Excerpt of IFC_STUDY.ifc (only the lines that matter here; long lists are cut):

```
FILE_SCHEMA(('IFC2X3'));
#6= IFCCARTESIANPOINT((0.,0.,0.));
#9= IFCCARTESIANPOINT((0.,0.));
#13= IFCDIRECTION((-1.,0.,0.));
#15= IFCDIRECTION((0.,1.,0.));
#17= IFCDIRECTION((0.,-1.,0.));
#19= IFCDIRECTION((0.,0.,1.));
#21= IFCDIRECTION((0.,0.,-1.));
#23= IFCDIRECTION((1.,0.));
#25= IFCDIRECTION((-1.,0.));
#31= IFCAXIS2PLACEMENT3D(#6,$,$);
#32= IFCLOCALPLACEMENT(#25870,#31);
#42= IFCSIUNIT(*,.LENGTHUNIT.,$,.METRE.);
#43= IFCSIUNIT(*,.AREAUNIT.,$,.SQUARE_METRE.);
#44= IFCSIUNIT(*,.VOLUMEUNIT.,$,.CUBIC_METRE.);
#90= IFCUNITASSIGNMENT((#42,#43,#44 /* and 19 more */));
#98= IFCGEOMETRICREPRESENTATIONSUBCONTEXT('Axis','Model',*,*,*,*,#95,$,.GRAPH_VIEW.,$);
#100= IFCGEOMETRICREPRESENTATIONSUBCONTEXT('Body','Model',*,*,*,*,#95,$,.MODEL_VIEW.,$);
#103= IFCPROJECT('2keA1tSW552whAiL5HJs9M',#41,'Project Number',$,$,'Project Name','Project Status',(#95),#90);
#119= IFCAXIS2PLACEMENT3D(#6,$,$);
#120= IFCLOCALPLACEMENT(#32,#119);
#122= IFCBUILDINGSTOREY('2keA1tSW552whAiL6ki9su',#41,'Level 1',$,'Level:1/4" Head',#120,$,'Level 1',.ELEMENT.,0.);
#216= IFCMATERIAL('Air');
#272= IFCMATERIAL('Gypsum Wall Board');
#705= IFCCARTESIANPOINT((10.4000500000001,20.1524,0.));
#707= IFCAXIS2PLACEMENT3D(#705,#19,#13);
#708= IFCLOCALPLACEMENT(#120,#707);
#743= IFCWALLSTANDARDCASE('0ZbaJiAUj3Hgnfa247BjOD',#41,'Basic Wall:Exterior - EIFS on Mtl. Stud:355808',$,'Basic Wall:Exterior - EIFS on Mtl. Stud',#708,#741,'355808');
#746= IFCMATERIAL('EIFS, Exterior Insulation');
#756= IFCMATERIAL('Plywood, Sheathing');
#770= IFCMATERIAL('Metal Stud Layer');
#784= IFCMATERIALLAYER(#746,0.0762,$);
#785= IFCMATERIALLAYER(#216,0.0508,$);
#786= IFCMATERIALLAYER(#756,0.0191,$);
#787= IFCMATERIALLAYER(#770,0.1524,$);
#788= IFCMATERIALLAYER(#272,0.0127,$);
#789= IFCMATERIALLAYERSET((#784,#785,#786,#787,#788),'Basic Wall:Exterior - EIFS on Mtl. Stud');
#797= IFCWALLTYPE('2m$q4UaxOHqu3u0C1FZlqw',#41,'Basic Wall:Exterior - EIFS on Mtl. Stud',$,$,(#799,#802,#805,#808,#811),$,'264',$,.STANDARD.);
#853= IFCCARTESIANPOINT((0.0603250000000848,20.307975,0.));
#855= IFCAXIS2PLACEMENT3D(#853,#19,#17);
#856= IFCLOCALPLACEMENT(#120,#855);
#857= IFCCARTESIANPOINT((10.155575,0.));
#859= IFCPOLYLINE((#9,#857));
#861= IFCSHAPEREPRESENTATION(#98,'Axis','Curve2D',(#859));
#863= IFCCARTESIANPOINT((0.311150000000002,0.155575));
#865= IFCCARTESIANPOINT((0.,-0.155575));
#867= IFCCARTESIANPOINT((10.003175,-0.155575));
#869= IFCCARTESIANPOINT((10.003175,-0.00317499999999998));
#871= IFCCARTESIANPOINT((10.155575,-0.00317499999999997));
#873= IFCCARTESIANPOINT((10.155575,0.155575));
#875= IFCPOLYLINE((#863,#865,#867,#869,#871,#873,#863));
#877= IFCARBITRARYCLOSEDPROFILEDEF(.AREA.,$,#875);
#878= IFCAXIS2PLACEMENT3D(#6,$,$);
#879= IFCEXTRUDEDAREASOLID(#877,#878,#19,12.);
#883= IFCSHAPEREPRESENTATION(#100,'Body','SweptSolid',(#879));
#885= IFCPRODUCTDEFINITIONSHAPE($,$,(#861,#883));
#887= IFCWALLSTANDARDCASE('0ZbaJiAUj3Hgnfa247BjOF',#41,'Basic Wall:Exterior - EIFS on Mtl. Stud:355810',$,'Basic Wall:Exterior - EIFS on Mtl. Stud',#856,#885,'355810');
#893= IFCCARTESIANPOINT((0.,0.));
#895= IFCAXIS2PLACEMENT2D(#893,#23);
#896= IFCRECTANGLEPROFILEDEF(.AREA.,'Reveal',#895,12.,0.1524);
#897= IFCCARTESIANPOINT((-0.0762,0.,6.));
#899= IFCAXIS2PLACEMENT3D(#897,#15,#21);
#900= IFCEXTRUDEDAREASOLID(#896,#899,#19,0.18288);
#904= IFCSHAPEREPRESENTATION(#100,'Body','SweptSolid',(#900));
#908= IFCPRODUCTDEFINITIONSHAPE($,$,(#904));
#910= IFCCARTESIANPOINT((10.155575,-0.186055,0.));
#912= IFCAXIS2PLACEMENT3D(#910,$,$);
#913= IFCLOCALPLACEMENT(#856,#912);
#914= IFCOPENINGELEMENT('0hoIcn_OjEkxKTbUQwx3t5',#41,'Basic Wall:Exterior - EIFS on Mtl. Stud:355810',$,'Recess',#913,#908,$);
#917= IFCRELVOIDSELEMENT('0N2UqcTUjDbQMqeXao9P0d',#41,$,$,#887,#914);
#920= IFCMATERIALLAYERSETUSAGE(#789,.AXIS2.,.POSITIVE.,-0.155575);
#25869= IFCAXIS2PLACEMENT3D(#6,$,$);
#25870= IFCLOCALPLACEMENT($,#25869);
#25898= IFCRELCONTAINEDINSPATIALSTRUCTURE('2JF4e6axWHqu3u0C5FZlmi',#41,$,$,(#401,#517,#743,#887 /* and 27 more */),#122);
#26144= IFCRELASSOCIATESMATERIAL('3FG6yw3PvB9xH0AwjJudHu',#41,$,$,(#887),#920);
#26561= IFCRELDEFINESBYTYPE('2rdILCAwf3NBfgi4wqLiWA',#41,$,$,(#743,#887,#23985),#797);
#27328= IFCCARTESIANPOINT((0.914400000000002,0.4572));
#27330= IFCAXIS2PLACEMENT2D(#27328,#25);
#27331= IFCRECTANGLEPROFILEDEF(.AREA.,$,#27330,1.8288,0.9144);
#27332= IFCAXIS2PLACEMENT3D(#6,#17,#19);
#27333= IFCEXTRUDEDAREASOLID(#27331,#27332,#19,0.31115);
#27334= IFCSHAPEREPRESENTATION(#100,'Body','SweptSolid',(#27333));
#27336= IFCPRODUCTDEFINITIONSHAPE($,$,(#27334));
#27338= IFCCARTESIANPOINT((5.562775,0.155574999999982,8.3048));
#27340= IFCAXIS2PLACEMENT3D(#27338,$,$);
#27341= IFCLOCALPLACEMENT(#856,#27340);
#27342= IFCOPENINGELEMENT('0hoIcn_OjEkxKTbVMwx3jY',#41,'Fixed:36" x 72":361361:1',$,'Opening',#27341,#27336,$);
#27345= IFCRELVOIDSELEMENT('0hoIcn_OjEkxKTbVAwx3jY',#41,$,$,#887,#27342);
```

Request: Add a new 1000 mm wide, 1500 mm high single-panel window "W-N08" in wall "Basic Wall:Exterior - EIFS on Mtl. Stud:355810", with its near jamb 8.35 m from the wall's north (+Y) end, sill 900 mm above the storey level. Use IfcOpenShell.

```python
import numpy as np
import ifcopenshell
import ifcopenshell.api.feature
import ifcopenshell.api.geometry
import ifcopenshell.api.root
import ifcopenshell.api.spatial
import ifcopenshell.api.type
import ifcopenshell.geom
import ifcopenshell.util.element
import ifcopenshell.util.placement
import ifcopenshell.util.representation
import ifcopenshell.util.shape
import ifcopenshell.util.unit

model = ifcopenshell.open("IFC_STUDY.ifc")
unit_scale = ifcopenshell.util.unit.calculate_unit_scale(model)
settings = ifcopenshell.geom.settings()


def volume(element):
    """Net volume in cubic metres, openings subtracted."""
    shape = ifcopenshell.geom.create_shape(settings, element)
    return ifcopenshell.util.shape.get_volume(shape.geometry)


wall = model.by_guid("0ZbaJiAUj3Hgnfa247BjOF")
storey = ifcopenshell.util.element.get_container(wall, ifc_class="IfcBuildingStorey")
context = ifcopenshell.util.representation.get_context(model, "Model", "Body", "MODEL_VIEW")
before = volume(wall)

width, height, from_end, sill = 1, 1.5, 8.35, 0.9  # metres

# The wall runs along its own X axis, and the end named is its -X end.
wall_shape = ifcopenshell.geom.create_shape(settings, wall)
x, y, z = ifcopenshell.util.shape.get_vertices(wall_shape.geometry).T
start = x.min() + from_end
face, thickness = float(y.min()), float(y.max() - y.min())
wall_matrix = ifcopenshell.util.placement.get_local_placement(wall.ObjectPlacement)
level = ifcopenshell.util.placement.get_local_placement(storey.ObjectPlacement)[2, 3]


def in_wall(x, y):
    """Placement at x, y metres in the wall's axes, at sill height."""
    matrix = wall_matrix.copy()
    matrix[:, 3] = wall_matrix @ np.array([x / unit_scale, y / unit_scale, 0.0, 1.0])
    matrix[2, 3] = level + sill / unit_scale
    return matrix


# Opening: a box that overshoots both wall faces by 50 mm.
opening = ifcopenshell.api.root.create_entity(model, ifc_class="IfcOpeningElement")
box = ifcopenshell.api.geometry.add_wall_representation(
    model, context=context, length=width, height=height, thickness=thickness + 0.1
)
ifcopenshell.api.geometry.assign_representation(model, product=opening, representation=box)
ifcopenshell.api.geometry.edit_object_placement(model, product=opening, matrix=in_wall(start, face - 0.05), is_si=False)
ifcopenshell.api.feature.add_feature(model, feature=opening, element=wall)

window = ifcopenshell.api.root.create_entity(model, ifc_class="IfcWindow", name="W-N08")
window.OverallWidth, window.OverallHeight = width / unit_scale, height / unit_scale
body = ifcopenshell.api.geometry.add_window_representation(
    model,
    context=context,
    overall_width=window.OverallWidth,
    overall_height=window.OverallHeight,
    partition_type="SINGLE_PANEL",
)
ifcopenshell.api.geometry.assign_representation(model, product=window, representation=body)
ifcopenshell.api.spatial.assign_container(model, products=[window], relating_structure=storey)
fills = ifcopenshell.api.feature.add_filling(model, opening=opening, element=window)
fills.OwnerHistory = window.OwnerHistory  # required in IFC2X3

# IFC2X3 keeps the operation on the window style.
style = ifcopenshell.api.root.create_entity(model, ifc_class="IfcWindowStyle", name="W-N08")
style.OperationType, style.ConstructionType = "SINGLE_PANEL", "NOTDEFINED"
style.ParameterTakesPrecedence = style.Sizeable = False
ifcopenshell.api.type.assign_type(model, related_objects=[window], relating_type=style)

# Centre the window in the wall's thickness.
ifcopenshell.api.geometry.edit_object_placement(model, product=window, matrix=in_wall(start, face), is_si=False)
window_shape = ifcopenshell.geom.create_shape(settings, window)
depth = ifcopenshell.util.shape.get_vertices(window_shape.geometry)[:, 1]
offset = face + thickness / 2 - (depth.min() + depth.max()) / 2
ifcopenshell.api.geometry.edit_object_placement(model, product=window, matrix=in_wall(start, offset), is_si=False)

after = volume(wall)

print(f"wall volume {before:.3f} -> {after:.3f} m3")

model.write("IFC_STUDY_edited.ifc")
```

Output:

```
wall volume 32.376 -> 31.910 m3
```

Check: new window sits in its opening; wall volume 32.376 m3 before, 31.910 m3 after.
